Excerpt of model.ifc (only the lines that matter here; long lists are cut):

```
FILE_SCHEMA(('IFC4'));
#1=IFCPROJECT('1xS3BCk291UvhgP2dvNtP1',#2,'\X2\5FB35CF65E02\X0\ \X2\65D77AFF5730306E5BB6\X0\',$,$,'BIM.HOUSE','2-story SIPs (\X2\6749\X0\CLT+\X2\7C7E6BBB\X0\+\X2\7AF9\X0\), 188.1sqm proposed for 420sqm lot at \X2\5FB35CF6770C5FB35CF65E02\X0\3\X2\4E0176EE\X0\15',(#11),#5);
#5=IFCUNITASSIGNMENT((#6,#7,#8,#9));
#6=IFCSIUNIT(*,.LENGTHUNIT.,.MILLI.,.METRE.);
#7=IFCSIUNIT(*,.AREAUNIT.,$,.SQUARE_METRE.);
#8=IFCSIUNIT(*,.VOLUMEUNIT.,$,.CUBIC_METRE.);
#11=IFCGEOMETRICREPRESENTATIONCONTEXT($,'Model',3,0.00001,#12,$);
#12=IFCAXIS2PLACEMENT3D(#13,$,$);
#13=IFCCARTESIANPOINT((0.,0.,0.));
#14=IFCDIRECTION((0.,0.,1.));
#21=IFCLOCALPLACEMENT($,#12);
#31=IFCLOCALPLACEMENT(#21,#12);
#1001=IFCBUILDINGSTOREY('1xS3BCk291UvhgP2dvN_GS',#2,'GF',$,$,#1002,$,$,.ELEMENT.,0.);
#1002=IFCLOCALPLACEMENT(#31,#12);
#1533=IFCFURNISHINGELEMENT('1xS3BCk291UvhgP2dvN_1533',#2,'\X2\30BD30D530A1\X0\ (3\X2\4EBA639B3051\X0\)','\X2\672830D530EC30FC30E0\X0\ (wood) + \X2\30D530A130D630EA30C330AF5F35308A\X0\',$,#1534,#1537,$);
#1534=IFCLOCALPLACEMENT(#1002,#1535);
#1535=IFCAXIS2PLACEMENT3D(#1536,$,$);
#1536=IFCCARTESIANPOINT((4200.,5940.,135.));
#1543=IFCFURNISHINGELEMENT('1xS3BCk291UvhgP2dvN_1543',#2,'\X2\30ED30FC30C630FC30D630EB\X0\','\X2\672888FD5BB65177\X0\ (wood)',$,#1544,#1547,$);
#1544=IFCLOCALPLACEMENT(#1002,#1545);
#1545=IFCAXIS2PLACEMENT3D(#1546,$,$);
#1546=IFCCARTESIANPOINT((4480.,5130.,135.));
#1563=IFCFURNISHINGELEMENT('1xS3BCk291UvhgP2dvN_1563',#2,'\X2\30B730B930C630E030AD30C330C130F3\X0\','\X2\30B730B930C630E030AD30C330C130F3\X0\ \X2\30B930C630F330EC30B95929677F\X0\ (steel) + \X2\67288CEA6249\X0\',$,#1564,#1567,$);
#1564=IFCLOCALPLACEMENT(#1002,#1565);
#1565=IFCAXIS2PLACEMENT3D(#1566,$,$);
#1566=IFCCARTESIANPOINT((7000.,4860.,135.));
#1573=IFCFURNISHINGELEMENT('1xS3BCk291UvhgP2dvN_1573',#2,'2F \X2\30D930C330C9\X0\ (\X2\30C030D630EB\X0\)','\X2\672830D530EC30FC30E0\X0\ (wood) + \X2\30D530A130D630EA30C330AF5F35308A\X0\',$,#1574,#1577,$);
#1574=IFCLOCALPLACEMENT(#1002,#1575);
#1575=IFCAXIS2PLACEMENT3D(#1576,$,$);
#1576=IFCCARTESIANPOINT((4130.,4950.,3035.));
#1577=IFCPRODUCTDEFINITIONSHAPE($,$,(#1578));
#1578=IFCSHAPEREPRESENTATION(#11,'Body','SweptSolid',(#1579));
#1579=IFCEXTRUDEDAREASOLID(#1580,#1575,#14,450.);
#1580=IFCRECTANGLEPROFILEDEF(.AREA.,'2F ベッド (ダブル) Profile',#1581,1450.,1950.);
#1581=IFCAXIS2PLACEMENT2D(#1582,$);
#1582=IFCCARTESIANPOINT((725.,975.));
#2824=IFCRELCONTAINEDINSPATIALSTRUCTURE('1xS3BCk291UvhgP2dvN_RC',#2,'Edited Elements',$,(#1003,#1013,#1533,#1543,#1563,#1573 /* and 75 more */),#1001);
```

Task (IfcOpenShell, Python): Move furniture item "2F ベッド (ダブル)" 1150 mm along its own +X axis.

```python
import ifcopenshell
import ifcopenshell.api.geometry
import ifcopenshell.util.placement
import ifcopenshell.util.unit

model = ifcopenshell.open("model.ifc")
unit_scale = ifcopenshell.util.unit.calculate_unit_scale(model)

item = model.by_guid("1xS3BCk291UvhgP2dvN_1573")
matrix = ifcopenshell.util.placement.get_local_placement(item.ObjectPlacement)
matrix[:3, 3] += matrix[:3, 0] * 1.15 / unit_scale
ifcopenshell.api.geometry.edit_object_placement(model, product=item, matrix=matrix, is_si=False)

print(ifcopenshell.util.placement.get_local_placement(item.ObjectPlacement).round(3) + 0.0)

model.write("model-out.ifc")
```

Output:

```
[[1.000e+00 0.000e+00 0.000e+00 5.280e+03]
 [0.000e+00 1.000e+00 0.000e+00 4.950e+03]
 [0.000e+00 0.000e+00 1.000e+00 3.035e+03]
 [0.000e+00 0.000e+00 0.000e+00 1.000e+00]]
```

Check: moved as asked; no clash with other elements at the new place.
